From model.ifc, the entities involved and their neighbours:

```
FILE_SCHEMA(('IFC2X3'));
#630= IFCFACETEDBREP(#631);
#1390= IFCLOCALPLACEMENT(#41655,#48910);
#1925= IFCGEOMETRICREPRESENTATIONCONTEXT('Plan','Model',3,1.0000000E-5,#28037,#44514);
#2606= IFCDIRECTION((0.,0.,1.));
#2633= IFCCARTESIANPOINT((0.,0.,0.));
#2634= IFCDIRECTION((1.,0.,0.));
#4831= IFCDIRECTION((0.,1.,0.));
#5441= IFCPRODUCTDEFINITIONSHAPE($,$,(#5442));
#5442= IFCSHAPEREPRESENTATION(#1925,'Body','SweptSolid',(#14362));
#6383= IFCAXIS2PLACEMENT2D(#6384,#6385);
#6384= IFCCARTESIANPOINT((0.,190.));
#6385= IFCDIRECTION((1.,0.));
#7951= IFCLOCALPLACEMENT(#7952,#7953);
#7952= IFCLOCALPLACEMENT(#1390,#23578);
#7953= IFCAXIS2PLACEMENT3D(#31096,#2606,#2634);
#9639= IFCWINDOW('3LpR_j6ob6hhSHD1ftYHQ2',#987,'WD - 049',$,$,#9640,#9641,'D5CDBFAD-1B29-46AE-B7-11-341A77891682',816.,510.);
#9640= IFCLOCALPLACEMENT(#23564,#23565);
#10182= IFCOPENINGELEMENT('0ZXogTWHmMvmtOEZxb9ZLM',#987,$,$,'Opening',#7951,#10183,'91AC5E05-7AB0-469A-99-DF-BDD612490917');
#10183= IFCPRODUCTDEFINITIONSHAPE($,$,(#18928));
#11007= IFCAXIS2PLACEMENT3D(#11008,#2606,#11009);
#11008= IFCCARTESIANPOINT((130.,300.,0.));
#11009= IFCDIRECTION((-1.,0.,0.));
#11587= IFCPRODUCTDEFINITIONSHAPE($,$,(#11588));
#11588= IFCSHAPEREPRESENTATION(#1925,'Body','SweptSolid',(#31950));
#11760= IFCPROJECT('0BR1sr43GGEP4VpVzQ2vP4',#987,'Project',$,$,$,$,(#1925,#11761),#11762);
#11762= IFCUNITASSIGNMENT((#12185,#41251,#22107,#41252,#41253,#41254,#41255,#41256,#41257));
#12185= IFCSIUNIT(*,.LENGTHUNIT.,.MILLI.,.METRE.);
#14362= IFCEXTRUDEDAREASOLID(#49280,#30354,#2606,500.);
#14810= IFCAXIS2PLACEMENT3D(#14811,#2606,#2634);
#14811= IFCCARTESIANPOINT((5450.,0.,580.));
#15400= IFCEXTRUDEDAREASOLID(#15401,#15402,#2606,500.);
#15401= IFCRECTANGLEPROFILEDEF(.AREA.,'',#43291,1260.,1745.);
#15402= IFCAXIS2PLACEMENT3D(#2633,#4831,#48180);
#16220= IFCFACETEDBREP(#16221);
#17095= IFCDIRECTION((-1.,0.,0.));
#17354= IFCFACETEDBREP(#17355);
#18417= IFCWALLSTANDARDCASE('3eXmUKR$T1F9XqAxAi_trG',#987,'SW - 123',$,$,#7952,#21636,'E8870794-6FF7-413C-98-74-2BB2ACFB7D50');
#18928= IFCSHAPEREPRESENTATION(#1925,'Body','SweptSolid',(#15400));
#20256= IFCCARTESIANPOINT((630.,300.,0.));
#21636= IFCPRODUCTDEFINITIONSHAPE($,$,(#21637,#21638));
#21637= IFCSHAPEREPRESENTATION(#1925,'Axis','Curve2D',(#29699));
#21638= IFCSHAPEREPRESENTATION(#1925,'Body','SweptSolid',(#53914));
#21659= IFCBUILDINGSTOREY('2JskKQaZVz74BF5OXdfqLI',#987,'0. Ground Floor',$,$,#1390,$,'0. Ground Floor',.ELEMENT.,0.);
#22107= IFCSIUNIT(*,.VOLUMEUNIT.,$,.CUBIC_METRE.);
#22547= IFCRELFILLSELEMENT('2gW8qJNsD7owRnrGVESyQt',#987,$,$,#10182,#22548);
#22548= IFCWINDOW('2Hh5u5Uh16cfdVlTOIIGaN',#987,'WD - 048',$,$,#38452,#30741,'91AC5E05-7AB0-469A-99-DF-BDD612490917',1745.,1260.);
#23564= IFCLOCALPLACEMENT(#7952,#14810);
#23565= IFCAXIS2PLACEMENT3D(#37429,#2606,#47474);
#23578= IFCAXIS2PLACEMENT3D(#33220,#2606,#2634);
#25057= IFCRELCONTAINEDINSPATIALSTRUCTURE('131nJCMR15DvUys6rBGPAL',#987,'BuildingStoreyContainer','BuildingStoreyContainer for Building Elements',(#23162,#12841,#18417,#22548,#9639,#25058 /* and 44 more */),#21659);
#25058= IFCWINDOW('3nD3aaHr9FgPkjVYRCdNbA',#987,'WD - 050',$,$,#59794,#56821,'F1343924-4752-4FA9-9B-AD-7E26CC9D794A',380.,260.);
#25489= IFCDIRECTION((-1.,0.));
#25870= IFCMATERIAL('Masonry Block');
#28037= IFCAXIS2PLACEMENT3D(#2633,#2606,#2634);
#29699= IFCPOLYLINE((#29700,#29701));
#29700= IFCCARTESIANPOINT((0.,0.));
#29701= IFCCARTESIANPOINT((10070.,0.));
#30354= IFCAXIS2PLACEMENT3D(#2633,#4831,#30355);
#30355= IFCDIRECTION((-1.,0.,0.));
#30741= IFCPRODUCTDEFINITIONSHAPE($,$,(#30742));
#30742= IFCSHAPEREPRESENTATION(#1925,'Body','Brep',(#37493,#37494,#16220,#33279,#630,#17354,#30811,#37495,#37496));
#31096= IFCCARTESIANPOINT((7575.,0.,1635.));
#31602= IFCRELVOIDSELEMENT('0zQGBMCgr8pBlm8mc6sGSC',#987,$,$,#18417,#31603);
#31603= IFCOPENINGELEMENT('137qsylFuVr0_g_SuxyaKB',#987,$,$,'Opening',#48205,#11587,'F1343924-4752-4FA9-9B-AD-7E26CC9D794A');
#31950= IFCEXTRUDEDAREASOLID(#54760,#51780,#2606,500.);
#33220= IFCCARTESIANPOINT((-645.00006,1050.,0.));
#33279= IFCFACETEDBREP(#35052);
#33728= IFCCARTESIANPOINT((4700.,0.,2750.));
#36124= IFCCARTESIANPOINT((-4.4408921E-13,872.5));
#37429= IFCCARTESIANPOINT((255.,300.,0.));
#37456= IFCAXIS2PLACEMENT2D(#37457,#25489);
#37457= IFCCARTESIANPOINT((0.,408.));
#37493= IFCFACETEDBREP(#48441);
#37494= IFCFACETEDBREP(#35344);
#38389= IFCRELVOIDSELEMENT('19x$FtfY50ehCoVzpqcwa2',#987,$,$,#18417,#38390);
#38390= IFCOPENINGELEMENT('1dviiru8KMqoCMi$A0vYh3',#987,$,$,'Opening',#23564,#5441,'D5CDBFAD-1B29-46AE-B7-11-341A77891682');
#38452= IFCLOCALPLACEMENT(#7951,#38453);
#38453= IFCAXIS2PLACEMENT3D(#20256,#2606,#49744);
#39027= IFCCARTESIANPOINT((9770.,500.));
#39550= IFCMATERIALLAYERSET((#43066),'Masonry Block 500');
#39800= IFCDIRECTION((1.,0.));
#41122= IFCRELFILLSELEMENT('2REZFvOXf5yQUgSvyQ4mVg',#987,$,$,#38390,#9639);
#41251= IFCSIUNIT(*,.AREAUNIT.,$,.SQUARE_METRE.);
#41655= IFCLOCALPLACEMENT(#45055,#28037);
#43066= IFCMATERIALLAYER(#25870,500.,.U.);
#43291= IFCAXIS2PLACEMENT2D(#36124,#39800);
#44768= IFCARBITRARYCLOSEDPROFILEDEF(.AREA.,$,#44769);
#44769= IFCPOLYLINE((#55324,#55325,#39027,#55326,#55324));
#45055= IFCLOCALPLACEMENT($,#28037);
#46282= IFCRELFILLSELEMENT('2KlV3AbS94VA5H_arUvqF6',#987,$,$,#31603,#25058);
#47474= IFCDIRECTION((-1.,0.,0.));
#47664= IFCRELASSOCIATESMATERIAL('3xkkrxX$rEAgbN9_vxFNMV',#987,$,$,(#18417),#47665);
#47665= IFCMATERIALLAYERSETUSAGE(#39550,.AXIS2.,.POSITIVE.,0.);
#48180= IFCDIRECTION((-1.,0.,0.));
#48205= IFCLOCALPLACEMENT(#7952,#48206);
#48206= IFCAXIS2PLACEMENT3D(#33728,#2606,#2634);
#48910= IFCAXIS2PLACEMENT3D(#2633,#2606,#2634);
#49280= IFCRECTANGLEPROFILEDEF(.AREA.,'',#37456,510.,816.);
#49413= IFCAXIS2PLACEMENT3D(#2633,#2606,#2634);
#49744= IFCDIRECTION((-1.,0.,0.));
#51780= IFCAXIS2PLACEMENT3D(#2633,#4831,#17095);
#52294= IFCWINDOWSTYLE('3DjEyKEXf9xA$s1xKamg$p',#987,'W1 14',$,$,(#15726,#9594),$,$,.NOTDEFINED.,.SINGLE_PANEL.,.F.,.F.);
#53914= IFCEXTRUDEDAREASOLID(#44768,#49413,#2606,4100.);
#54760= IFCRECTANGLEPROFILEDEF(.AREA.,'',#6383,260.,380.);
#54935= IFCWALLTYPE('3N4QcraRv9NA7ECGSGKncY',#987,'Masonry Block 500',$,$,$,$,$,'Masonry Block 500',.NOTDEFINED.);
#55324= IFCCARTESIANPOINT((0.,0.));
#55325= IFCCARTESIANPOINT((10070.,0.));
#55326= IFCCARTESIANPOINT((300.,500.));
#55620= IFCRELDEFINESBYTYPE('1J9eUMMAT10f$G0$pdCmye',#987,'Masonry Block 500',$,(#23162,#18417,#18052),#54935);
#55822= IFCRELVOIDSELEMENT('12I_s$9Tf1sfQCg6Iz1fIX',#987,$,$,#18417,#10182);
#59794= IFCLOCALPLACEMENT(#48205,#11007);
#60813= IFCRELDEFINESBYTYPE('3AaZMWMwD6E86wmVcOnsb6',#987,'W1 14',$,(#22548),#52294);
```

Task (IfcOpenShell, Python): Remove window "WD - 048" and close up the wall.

```python
import ifcopenshell
import ifcopenshell.api.feature
import ifcopenshell.api.root
import ifcopenshell.geom
import ifcopenshell.util.shape

model = ifcopenshell.open("model.ifc")
settings = ifcopenshell.geom.settings()


def volume(element):
    """Net volume in cubic metres, openings subtracted."""
    shape = ifcopenshell.geom.create_shape(settings, element)
    return ifcopenshell.util.shape.get_volume(shape.geometry)


window = model.by_id(22548)
opening = window.FillsVoids[0].RelatingOpeningElement
wall = opening.VoidsElements[0].RelatingBuildingElement
before = volume(wall)

ifcopenshell.api.root.remove_product(model, product=window)
ifcopenshell.api.feature.remove_feature(model, feature=opening)

after = volume(wall)

print(f"wall volume {before:.3f} -> {after:.3f} m3")

model.write("model_updated.ifc")
```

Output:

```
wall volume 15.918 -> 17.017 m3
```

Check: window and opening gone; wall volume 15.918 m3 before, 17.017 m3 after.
